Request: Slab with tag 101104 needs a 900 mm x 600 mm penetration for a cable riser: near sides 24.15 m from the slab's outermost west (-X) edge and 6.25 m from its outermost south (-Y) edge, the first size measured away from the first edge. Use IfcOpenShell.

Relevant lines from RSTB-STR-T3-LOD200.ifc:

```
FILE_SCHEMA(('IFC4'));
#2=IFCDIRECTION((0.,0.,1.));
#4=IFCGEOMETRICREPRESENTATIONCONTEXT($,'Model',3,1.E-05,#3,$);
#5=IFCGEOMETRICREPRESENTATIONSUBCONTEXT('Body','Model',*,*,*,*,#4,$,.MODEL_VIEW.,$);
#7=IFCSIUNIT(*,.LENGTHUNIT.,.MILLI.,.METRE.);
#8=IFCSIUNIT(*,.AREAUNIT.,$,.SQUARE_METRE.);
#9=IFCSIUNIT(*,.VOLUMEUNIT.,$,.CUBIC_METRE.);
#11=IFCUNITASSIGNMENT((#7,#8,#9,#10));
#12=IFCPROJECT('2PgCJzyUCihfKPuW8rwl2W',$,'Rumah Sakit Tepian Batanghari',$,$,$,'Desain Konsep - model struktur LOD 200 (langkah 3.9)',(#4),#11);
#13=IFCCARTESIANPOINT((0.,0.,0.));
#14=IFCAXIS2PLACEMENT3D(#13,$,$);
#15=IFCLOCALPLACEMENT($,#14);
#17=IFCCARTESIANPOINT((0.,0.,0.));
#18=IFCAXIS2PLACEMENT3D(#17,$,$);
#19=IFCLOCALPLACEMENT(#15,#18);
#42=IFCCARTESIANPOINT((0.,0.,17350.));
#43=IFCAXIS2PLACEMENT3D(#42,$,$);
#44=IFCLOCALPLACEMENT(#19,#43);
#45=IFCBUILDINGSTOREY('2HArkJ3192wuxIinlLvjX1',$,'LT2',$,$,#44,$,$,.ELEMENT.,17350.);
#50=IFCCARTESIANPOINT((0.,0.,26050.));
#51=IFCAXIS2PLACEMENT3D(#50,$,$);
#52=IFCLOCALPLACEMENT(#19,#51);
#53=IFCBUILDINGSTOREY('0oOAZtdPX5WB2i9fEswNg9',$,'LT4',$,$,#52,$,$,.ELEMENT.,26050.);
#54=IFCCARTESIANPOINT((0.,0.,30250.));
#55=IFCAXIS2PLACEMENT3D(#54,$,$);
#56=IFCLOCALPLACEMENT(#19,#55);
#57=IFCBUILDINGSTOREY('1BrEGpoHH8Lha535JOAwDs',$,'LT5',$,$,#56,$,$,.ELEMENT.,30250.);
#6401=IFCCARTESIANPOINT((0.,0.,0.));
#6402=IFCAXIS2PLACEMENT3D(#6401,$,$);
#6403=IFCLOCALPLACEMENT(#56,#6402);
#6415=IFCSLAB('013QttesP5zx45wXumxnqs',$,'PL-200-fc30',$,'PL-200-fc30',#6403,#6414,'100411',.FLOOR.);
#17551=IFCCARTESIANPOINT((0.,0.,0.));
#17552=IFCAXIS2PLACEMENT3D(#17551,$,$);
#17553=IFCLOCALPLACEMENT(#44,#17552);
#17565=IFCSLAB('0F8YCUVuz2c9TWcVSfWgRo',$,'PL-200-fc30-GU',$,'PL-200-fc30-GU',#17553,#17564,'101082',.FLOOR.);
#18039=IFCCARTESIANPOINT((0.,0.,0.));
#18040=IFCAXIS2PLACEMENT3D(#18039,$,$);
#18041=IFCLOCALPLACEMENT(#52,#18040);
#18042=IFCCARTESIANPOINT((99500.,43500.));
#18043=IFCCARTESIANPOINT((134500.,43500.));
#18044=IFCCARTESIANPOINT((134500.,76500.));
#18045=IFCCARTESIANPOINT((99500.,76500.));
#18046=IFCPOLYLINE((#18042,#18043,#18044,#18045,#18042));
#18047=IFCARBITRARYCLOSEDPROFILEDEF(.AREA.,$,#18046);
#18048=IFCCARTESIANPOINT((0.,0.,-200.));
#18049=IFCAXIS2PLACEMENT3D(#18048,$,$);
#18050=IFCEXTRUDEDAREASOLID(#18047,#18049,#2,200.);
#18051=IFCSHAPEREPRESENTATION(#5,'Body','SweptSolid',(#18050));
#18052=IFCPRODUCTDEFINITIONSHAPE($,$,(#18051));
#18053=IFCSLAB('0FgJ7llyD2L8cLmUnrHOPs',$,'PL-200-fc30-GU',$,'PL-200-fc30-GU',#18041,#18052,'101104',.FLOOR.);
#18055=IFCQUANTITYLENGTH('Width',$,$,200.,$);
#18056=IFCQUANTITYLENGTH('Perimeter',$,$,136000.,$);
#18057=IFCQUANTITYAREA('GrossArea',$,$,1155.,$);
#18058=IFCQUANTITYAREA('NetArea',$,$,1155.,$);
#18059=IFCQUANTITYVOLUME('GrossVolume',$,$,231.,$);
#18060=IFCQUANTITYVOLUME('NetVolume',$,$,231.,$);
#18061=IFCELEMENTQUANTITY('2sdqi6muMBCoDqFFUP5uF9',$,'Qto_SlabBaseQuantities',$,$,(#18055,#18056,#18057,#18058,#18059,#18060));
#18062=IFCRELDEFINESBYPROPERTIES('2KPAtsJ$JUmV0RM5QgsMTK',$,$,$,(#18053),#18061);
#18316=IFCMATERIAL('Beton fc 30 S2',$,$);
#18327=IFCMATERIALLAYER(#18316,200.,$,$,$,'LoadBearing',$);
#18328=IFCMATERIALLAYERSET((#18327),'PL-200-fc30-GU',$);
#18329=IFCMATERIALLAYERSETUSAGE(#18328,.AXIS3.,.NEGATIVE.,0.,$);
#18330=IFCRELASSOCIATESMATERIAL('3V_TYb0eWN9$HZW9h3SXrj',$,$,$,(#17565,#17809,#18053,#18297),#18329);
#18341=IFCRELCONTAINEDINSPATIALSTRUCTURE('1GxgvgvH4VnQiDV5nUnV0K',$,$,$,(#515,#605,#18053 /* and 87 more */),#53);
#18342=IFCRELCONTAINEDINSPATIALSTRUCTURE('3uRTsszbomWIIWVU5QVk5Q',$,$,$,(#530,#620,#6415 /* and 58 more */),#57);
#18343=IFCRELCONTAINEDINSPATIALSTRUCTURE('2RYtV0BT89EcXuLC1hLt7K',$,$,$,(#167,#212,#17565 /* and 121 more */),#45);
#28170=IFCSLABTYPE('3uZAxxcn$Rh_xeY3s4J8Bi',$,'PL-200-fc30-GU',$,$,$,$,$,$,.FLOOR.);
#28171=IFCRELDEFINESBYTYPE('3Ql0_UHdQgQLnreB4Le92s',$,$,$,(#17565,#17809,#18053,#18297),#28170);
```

```python
import numpy as np
import ifcopenshell
import ifcopenshell.api.feature
import ifcopenshell.api.geometry
import ifcopenshell.api.pset
import ifcopenshell.api.root
import ifcopenshell.geom
import ifcopenshell.util.element
import ifcopenshell.util.placement
import ifcopenshell.util.representation
import ifcopenshell.util.shape
import ifcopenshell.util.unit

model = ifcopenshell.open("RSTB-STR-T3-LOD200.ifc")
unit_scale = ifcopenshell.util.unit.calculate_unit_scale(model)
area_scale = ifcopenshell.util.unit.calculate_unit_scale(model, "AREAUNIT")
volume_scale = ifcopenshell.util.unit.calculate_unit_scale(model, "VOLUMEUNIT")
settings = ifcopenshell.geom.settings()


def volume(element):
    """Net volume in cubic metres, openings subtracted."""
    shape = ifcopenshell.geom.create_shape(settings, element)
    return ifcopenshell.util.shape.get_volume(shape.geometry)


slab = model.by_guid("0FgJ7llyD2L8cLmUnrHOPs")
before = volume(slab)

# Extent in the slab's own axes, in metres. The edges named are its -X and -Y sides.
slab_shape = ifcopenshell.geom.create_shape(settings, slab)
vertices = ifcopenshell.util.shape.get_vertices(slab_shape.geometry)
x_min, y_min, bottom = vertices.min(axis=0)
top = vertices[:, 2].max()

opening = ifcopenshell.api.root.create_entity(model, ifc_class="IfcOpeningElement", name="Cable riser opening", predefined_type="OPENING")
context = ifcopenshell.util.representation.get_context(model, "Model", "Body", "MODEL_VIEW")
width, depth = 0.9, 0.6
outline = [(0.0, 0.0), (width, 0.0), (width, depth), (0.0, depth), (0.0, 0.0)]
# Overshoot both faces by 50 mm so the cut is clean.
shape = ifcopenshell.api.geometry.add_slab_representation(
    model, context=context, depth=top - bottom + 0.1, polyline=outline
)
ifcopenshell.api.geometry.assign_representation(model, product=opening, representation=shape)

matrix = ifcopenshell.util.placement.get_local_placement(slab.ObjectPlacement)
matrix[:, 3] = matrix @ np.append(np.array([x_min + 24.15, y_min + 6.25, bottom - 0.05]) / unit_scale, 1.0)
ifcopenshell.api.geometry.edit_object_placement(model, product=opening, matrix=matrix, is_si=False)
ifcopenshell.api.feature.add_feature(model, feature=opening, element=slab)

after = volume(slab)

# Update the slab's stored quantities.
qto = model.by_id(ifcopenshell.util.element.get_pset(slab, "Qto_SlabBaseQuantities", should_inherit=False)["id"])
ifcopenshell.api.pset.edit_qto(model, qto=qto, properties={
    "NetArea": after / (top - bottom) / area_scale,
    "NetVolume": after / volume_scale,
})

print(f"slab volume {before:.3f} -> {after:.3f} m3")

model.write("RSTB-STR-T3-LOD200_v2.ifc")
```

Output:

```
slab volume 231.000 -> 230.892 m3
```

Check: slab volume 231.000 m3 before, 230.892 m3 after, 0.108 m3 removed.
